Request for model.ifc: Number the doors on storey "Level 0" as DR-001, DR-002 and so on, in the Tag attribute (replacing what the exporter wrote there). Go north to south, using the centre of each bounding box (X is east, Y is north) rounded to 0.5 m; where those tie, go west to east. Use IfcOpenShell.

First a look at what the model holds.

```python
import ifcopenshell
import ifcopenshell.util.element
import ifcopenshell.util.placement

model = ifcopenshell.open("model.ifc")
print(model.schema)
storey = next(s for s in model.by_type("IfcBuildingStorey") if s.Name == "Level 0")
doors = [e for e in ifcopenshell.util.element.get_decomposition(storey) if e.is_a("IfcDoor")]
for e in sorted(doors, key=lambda e: e.id()):
    origin = ifcopenshell.util.placement.get_local_placement(e.ObjectPlacement)[:3, 3]
    print(e.id(), e.Tag, e.Name, origin.round(2) + 0.0, sep=" | ")
```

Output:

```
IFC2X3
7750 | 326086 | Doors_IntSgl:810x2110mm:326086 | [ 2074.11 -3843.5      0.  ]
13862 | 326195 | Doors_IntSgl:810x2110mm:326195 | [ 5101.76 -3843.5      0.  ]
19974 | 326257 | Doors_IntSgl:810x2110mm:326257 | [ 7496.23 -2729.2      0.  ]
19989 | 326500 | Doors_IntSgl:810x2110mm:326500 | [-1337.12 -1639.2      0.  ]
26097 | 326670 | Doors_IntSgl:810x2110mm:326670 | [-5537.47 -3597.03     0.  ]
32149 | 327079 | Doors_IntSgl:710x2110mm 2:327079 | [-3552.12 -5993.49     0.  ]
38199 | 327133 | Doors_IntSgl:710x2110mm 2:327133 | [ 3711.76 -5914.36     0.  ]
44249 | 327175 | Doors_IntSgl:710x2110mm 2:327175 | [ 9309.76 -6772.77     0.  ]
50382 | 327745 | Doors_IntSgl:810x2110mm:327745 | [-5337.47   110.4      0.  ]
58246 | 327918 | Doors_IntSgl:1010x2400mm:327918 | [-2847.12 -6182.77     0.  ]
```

```python
import ifcopenshell
import ifcopenshell.geom
import ifcopenshell.util.element
import ifcopenshell.util.shape

model = ifcopenshell.open("model.ifc")
settings = ifcopenshell.geom.settings()
settings.set("use-world-coords", True)


def centre(element):
    shape = ifcopenshell.geom.create_shape(settings, element)
    return ifcopenshell.util.shape.get_bbox_centroid(shape.geometry)


storey = next(s for s in model.by_type("IfcBuildingStorey") if s.Name == "Level 0")
doors = [e for e in ifcopenshell.util.element.get_decomposition(storey) if e.is_a("IfcDoor")]

# Insertion points can sit at a corner or the storey origin, so sort by the geometry (in metres).
centres = {e: centre(e) for e in doors}
doors.sort(key=lambda e: (-round(centres[e][1] / 0.5), centres[e][0]))

for i, e in enumerate(doors, start=1):
    number = f"DR-0{i:02d}"
    e.Tag = number
    print(e.id(), number)

model.write("model_edited.ifc")
```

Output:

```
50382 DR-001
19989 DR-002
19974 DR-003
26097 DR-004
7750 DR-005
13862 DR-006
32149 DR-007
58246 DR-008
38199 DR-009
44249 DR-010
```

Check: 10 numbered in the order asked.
